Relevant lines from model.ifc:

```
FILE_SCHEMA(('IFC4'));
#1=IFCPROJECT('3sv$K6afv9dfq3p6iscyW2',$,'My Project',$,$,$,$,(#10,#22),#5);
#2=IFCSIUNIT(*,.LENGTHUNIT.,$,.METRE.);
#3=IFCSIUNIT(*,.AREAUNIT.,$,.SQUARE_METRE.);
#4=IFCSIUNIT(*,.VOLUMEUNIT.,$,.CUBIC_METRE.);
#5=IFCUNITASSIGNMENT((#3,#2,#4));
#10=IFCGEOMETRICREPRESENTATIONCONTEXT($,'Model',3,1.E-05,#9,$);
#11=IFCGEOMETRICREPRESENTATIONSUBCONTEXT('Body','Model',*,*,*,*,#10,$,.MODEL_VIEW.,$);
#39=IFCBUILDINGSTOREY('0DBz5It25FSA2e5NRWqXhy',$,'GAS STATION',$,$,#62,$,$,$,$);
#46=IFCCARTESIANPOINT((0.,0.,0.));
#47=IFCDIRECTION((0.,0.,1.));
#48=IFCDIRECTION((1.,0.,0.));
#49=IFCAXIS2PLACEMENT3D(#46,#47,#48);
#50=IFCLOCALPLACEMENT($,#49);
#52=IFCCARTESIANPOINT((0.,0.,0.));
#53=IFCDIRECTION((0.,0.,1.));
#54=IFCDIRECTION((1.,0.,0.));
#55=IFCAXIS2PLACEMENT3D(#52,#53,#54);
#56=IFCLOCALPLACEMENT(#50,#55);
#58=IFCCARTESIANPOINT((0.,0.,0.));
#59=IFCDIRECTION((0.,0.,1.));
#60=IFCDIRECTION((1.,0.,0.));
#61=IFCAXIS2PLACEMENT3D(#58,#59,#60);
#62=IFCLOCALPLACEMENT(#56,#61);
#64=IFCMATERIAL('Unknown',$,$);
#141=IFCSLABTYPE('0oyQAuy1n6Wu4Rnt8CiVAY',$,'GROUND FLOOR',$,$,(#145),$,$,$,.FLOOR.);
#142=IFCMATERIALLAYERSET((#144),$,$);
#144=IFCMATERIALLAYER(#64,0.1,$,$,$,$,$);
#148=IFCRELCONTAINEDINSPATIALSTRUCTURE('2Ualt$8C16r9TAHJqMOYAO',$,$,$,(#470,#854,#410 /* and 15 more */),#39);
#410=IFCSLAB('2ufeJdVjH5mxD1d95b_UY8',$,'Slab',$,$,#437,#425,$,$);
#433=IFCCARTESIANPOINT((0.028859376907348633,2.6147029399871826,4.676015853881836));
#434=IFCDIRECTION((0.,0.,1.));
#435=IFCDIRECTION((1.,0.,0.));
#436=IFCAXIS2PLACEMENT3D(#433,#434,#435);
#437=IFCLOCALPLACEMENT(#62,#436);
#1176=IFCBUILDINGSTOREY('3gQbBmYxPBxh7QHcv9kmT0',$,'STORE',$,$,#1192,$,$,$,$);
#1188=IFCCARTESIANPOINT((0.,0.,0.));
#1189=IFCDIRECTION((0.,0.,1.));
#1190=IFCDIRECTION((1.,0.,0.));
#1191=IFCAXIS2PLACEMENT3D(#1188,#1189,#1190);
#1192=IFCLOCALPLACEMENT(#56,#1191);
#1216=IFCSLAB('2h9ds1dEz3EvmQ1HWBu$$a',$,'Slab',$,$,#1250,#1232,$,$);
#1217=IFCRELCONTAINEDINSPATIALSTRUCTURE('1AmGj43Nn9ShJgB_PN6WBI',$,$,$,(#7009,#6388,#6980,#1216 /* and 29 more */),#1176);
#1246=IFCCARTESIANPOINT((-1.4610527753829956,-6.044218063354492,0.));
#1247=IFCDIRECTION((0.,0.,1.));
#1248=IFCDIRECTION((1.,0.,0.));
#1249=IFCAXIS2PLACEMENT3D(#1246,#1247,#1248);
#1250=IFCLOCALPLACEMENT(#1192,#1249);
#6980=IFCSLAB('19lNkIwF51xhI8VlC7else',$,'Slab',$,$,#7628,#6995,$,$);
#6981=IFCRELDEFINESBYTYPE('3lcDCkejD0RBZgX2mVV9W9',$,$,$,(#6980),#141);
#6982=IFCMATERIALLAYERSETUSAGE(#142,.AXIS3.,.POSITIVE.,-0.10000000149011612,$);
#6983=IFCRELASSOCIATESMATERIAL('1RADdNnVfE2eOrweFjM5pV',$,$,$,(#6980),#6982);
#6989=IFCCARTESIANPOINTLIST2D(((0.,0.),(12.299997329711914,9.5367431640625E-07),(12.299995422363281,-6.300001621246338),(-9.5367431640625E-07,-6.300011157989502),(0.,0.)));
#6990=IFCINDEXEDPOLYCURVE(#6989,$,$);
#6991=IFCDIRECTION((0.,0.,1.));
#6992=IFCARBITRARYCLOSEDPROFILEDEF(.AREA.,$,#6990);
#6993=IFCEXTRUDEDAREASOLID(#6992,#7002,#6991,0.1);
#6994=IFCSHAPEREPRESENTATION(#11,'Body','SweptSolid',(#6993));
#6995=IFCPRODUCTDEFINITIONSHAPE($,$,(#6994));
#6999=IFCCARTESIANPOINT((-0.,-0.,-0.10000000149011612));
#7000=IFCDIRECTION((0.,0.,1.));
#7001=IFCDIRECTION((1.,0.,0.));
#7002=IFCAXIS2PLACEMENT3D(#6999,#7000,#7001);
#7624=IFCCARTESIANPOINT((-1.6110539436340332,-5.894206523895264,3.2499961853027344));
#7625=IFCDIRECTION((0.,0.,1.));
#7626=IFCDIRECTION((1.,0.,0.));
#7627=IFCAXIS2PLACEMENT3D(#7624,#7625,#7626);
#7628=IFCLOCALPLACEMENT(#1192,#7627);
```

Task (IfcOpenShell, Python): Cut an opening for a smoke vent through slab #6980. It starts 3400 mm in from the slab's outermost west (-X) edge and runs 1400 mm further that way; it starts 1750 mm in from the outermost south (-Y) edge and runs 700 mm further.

```python
import numpy as np
import ifcopenshell
import ifcopenshell.api.feature
import ifcopenshell.api.geometry
import ifcopenshell.api.root
import ifcopenshell.geom
import ifcopenshell.util.placement
import ifcopenshell.util.representation
import ifcopenshell.util.shape
import ifcopenshell.util.unit

model = ifcopenshell.open("model.ifc")
unit_scale = ifcopenshell.util.unit.calculate_unit_scale(model)
settings = ifcopenshell.geom.settings()


def volume(element):
    """Net volume in cubic metres, openings subtracted."""
    shape = ifcopenshell.geom.create_shape(settings, element)
    return ifcopenshell.util.shape.get_volume(shape.geometry)


slab = model.by_guid("19lNkIwF51xhI8VlC7else")
before = volume(slab)

# Extent in the slab's own axes, in metres. The edges named are its -X and -Y sides.
slab_shape = ifcopenshell.geom.create_shape(settings, slab)
vertices = ifcopenshell.util.shape.get_vertices(slab_shape.geometry)
x_min, y_min, bottom = vertices.min(axis=0)
top = vertices[:, 2].max()

opening = ifcopenshell.api.root.create_entity(model, ifc_class="IfcOpeningElement", name="Smoke vent opening", predefined_type="OPENING")
context = ifcopenshell.util.representation.get_context(model, "Model", "Body", "MODEL_VIEW")
width, depth = 1.4, 0.7
outline = [(0.0, 0.0), (width, 0.0), (width, depth), (0.0, depth), (0.0, 0.0)]
# Overshoot both faces by 50 mm so the cut is clean.
shape = ifcopenshell.api.geometry.add_slab_representation(
    model, context=context, depth=top - bottom + 0.1, polyline=outline
)
ifcopenshell.api.geometry.assign_representation(model, product=opening, representation=shape)

matrix = ifcopenshell.util.placement.get_local_placement(slab.ObjectPlacement)
matrix[:, 3] = matrix @ np.append(np.array([x_min + 3.4, y_min + 1.75, bottom - 0.05]) / unit_scale, 1.0)
ifcopenshell.api.geometry.edit_object_placement(model, product=opening, matrix=matrix, is_si=False)
ifcopenshell.api.feature.add_feature(model, feature=opening, element=slab)

after = volume(slab)

print(f"slab volume {before:.3f} -> {after:.3f} m3")

model.write("model-out.ifc")
```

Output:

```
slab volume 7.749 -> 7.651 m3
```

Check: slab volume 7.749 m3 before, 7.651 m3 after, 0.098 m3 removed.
